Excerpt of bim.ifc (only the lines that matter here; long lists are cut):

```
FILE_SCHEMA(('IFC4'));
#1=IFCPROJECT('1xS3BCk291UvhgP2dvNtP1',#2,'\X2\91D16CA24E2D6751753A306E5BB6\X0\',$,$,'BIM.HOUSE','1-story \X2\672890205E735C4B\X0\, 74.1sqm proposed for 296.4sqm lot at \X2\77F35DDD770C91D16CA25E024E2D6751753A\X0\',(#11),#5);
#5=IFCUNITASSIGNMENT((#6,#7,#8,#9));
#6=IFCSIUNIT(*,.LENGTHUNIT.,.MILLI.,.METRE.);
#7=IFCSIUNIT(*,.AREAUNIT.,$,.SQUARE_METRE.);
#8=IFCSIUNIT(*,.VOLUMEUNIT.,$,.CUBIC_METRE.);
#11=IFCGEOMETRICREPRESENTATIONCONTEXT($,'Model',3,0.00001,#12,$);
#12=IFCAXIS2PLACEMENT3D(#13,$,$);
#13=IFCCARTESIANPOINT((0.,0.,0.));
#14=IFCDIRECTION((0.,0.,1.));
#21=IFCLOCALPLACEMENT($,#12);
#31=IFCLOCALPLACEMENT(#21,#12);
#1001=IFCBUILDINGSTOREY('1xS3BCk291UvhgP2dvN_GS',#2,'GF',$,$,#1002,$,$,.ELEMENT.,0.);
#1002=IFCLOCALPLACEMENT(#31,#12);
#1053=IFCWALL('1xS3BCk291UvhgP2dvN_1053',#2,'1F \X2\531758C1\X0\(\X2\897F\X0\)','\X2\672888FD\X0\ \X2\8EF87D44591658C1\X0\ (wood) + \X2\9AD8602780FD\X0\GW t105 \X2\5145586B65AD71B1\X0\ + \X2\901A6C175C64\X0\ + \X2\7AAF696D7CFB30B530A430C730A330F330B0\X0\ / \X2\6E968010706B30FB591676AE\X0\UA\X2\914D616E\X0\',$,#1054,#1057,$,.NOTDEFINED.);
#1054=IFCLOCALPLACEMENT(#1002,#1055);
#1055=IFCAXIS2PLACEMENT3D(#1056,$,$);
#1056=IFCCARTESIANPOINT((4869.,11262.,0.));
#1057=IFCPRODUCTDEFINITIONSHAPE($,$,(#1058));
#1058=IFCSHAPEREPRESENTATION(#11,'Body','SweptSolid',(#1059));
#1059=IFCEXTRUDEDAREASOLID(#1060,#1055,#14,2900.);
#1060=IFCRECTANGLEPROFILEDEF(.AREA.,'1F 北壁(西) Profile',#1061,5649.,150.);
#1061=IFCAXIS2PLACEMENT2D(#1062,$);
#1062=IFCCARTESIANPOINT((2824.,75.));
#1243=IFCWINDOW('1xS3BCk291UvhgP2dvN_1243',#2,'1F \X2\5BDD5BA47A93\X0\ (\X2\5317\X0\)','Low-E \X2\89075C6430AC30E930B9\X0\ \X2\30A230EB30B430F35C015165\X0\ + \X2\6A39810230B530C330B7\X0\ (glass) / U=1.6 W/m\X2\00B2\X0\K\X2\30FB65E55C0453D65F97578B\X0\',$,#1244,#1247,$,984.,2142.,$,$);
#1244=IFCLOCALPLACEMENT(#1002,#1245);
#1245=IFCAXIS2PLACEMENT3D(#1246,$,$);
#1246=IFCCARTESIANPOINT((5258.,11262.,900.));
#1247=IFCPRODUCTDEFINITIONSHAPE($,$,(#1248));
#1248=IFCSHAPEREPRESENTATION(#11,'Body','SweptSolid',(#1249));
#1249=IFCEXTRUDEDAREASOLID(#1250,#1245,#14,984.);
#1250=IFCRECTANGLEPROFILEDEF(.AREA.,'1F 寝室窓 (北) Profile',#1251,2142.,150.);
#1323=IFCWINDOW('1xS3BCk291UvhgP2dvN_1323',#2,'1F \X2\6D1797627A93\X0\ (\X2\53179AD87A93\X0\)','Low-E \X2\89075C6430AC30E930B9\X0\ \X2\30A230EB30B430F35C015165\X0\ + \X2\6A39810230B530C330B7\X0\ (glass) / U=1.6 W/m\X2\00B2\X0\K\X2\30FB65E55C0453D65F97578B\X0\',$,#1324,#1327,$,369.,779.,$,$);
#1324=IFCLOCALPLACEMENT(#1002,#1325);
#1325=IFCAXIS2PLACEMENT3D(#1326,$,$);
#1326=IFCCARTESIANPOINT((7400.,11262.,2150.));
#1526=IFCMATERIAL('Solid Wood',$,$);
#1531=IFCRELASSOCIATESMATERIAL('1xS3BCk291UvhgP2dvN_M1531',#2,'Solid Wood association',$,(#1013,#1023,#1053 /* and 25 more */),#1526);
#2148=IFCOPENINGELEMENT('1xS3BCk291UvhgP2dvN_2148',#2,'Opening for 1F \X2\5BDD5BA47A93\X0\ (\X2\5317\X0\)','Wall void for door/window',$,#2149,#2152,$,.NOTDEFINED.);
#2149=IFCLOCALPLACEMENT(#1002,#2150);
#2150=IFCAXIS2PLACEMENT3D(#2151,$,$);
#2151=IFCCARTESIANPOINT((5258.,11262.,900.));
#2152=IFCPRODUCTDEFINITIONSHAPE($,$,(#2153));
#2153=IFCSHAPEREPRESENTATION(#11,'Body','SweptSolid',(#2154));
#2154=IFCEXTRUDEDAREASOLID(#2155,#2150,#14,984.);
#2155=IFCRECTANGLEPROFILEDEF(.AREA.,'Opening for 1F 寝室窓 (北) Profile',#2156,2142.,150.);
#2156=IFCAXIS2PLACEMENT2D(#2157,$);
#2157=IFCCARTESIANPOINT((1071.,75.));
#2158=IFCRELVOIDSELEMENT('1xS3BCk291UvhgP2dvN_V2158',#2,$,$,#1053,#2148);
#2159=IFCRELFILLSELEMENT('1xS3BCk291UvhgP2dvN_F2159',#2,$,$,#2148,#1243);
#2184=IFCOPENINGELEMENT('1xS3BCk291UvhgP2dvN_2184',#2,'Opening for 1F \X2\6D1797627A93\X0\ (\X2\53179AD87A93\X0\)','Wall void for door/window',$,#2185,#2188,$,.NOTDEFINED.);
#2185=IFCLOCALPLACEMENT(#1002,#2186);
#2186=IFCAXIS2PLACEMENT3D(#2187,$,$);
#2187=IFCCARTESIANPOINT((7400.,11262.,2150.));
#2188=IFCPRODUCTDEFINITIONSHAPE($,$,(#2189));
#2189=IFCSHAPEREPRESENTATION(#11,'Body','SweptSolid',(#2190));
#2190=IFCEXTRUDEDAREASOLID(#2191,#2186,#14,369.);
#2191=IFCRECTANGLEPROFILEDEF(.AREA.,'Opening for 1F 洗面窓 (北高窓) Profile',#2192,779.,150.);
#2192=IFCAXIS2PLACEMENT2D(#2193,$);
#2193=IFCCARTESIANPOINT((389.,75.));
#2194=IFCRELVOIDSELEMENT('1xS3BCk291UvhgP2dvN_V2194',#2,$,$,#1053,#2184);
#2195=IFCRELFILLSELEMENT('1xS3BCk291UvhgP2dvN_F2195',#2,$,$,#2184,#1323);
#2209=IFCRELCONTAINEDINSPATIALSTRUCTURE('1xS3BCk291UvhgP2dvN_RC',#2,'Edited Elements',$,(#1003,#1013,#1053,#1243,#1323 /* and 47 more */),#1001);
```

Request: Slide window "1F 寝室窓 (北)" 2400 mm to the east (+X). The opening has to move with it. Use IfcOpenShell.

```python
import ifcopenshell
import ifcopenshell.api.geometry
import ifcopenshell.util.placement

model = ifcopenshell.open("bim.ifc")

window = model.by_id(1243)
opening = window.FillsVoids[0].RelatingOpeningElement
wall = opening.VoidsElements[0].RelatingBuildingElement

wall_matrix = ifcopenshell.util.placement.get_local_placement(wall.ObjectPlacement)
shift = wall_matrix[:3, 0] * 2400.0
before = ifcopenshell.util.placement.get_local_placement(window.ObjectPlacement)[:3, 3].copy()

# The window is not placed relative to its opening, so move both.
for product in (opening, window):
    matrix = ifcopenshell.util.placement.get_local_placement(product.ObjectPlacement)
    matrix[:3, 3] += shift
    ifcopenshell.api.geometry.edit_object_placement(model, product=product, matrix=matrix, is_si=False)

after = ifcopenshell.util.placement.get_local_placement(window.ObjectPlacement)[:3, 3]
print("window moved by", (after - before).round(3) + 0.0)

model.write("bim_v2.ifc")
```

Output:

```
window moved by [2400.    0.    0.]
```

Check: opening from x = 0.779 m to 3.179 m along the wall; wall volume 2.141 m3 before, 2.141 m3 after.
